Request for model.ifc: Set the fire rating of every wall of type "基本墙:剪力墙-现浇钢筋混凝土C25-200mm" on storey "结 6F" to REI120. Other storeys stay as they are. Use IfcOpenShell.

First a look at what the model holds.

```python
import ifcopenshell
import ifcopenshell.util.element

model = ifcopenshell.open("model.ifc")
print(model.schema)
storey = next(s for s in model.by_type("IfcBuildingStorey") if s.Name == "结 6F")
walls = [e for e in ifcopenshell.util.element.get_decomposition(storey) if e.is_a("IfcWall")]
seen = {}
for e in walls:
    element_type = ifcopenshell.util.element.get_type(e)
    key = (element_type.Name if element_type != e and element_type else None, ifcopenshell.util.element.get_pset(e, "Pset_WallCommon", "FireRating"))
    seen[key] = seen.get(key, 0) + 1
for (name, value), count in sorted(seen.items(), key=str):
    print(count, "x", name, "|", value)
```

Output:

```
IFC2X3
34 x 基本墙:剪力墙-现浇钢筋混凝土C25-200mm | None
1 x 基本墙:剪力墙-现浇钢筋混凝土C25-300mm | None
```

```python
import ifcopenshell
import ifcopenshell.api.pset
import ifcopenshell.util.element

model = ifcopenshell.open("model.ifc")

storey = next(s for s in model.by_type("IfcBuildingStorey") if s.Name == "结 6F")
walls = [e for e in ifcopenshell.util.element.get_decomposition(storey) if e.is_a("IfcWall")]

count = 0
for e in walls:
    element_type = ifcopenshell.util.element.get_type(e)
    if element_type in (None, e) or element_type.Name != "基本墙:剪力墙-现浇钢筋混凝土C25-200mm":
        continue
    # add_pset returns the element's existing set when there is one.
    pset = ifcopenshell.api.pset.add_pset(model, product=e, name="Pset_WallCommon")
    ifcopenshell.api.pset.edit_pset(model, pset=pset, properties={"FireRating": "REI120"})
    count += 1

print(count, "walls updated")

model.write("model-out.ifc")
```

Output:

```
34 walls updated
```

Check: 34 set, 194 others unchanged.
